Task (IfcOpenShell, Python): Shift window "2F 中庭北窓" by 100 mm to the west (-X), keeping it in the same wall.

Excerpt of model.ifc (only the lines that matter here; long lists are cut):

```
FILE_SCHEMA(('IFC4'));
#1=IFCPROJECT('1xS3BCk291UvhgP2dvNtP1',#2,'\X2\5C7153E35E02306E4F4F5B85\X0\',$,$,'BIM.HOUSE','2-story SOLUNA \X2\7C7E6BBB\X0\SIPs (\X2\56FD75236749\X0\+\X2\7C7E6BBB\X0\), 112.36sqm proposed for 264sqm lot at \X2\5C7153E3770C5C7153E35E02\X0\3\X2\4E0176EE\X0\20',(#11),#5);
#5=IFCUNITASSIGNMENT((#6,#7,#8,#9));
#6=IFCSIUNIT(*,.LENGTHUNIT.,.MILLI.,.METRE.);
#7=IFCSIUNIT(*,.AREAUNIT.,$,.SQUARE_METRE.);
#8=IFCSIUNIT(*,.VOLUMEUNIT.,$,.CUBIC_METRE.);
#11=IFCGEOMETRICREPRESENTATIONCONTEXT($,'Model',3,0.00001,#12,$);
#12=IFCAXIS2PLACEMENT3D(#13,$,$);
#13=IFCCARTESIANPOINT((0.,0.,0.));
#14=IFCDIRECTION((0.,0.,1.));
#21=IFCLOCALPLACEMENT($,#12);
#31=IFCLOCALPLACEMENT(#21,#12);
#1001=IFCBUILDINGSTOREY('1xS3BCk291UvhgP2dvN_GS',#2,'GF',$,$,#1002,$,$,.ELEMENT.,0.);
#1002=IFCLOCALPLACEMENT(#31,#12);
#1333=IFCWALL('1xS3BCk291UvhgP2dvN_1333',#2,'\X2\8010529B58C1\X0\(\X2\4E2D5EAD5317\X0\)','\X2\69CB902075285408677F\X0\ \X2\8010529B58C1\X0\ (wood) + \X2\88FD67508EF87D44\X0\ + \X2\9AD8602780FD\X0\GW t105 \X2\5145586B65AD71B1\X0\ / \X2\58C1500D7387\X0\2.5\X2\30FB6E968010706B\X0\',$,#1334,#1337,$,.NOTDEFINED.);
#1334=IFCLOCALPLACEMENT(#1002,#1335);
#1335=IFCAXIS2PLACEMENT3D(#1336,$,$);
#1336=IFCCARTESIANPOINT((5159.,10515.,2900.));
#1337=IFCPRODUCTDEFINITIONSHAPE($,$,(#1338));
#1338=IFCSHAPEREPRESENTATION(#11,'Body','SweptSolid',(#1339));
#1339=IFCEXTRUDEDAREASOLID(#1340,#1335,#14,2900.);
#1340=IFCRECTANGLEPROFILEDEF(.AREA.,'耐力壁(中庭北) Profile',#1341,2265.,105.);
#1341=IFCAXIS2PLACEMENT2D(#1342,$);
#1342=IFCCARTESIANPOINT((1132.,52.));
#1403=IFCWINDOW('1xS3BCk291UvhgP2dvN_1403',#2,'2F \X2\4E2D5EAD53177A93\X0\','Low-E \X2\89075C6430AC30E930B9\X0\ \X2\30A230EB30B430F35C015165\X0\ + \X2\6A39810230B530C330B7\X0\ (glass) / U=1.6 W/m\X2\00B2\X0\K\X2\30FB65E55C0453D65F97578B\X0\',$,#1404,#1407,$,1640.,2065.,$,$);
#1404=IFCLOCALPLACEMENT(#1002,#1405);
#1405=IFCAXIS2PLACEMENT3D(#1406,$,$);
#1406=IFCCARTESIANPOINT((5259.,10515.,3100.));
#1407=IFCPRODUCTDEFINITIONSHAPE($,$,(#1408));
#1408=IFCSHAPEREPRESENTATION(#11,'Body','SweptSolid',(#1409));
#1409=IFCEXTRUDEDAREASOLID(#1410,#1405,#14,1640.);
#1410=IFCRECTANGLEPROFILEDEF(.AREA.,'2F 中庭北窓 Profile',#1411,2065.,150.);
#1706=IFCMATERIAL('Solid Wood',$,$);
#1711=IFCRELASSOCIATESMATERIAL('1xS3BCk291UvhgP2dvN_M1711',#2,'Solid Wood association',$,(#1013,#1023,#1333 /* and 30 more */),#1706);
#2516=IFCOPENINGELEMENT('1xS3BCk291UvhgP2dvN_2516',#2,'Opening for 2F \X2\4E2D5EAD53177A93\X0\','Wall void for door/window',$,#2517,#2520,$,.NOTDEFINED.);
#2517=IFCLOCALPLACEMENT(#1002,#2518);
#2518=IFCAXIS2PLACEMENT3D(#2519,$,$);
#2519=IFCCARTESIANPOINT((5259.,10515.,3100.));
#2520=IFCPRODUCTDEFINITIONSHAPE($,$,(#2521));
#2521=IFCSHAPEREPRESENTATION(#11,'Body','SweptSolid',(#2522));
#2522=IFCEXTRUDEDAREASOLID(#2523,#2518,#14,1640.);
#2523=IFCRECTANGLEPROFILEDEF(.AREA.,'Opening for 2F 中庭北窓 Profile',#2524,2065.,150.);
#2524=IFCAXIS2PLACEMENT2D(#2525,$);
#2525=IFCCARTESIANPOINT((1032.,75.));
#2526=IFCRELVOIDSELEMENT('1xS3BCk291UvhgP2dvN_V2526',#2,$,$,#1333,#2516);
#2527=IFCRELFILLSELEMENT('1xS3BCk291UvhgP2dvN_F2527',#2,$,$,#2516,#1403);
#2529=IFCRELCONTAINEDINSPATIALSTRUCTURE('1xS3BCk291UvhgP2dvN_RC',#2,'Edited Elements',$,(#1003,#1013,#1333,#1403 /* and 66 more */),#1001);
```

```python
import ifcopenshell
import ifcopenshell.api.geometry
import ifcopenshell.util.placement
import ifcopenshell.util.unit

model = ifcopenshell.open("model.ifc")
unit_scale = ifcopenshell.util.unit.calculate_unit_scale(model)

window = model.by_guid("1xS3BCk291UvhgP2dvN_1403")
opening = window.FillsVoids[0].RelatingOpeningElement
wall = opening.VoidsElements[0].RelatingBuildingElement

wall_matrix = ifcopenshell.util.placement.get_local_placement(wall.ObjectPlacement)
shift = wall_matrix[:3, 0] * -0.1 / unit_scale
before = ifcopenshell.util.placement.get_local_placement(window.ObjectPlacement)[:3, 3].copy()

# The window is not placed relative to its opening, so move both.
for product in (opening, window):
    matrix = ifcopenshell.util.placement.get_local_placement(product.ObjectPlacement)
    matrix[:3, 3] += shift
    ifcopenshell.api.geometry.edit_object_placement(model, product=product, matrix=matrix, is_si=False)

after = ifcopenshell.util.placement.get_local_placement(window.ObjectPlacement)[:3, 3]
print("window moved by", (after - before).round(3) + 0.0)

model.write("model_rev.ifc")
```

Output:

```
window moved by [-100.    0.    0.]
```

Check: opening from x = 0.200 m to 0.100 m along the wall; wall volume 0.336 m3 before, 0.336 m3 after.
